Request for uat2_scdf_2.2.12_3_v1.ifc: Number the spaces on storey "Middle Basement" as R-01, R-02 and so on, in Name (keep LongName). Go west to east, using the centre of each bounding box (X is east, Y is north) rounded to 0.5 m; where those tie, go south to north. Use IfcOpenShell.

First a look at what the model holds.

```python
import ifcopenshell
import ifcopenshell.util.element
import ifcopenshell.util.placement

model = ifcopenshell.open("uat2_scdf_2.2.12_3_v1.ifc")
print(model.schema)
storey = next(s for s in model.by_type("IfcBuildingStorey") if s.Name == "Middle Basement")
spaces = [e for e in ifcopenshell.util.element.get_decomposition(storey) if e.is_a("IfcSpace")]
for e in sorted(spaces, key=lambda e: e.id()):
    origin = ifcopenshell.util.placement.get_local_placement(e.ObjectPlacement)[:3, 3]
    print(e.id(), e.Name, e.LongName, origin.round(2) + 0.0, sep=" | ")
```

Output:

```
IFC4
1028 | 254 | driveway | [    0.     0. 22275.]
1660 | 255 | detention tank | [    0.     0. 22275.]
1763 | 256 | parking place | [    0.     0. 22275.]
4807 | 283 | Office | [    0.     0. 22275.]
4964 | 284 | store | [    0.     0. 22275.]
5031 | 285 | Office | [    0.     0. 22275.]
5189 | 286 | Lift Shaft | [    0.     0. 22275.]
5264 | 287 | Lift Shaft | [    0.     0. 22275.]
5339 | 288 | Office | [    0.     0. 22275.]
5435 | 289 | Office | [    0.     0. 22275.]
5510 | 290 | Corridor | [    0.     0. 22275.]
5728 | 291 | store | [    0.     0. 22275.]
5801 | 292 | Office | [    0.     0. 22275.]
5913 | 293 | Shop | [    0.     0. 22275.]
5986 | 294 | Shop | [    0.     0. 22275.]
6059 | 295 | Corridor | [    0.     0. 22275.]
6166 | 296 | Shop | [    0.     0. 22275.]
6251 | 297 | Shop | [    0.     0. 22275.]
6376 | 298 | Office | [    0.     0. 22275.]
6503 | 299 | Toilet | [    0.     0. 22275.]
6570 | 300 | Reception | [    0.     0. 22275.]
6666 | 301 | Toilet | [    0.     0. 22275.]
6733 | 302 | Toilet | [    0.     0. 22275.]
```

```python
import ifcopenshell
import ifcopenshell.geom
import ifcopenshell.util.element
import ifcopenshell.util.shape

model = ifcopenshell.open("uat2_scdf_2.2.12_3_v1.ifc")
settings = ifcopenshell.geom.settings()
settings.set("use-world-coords", True)


def centre(element):
    shape = ifcopenshell.geom.create_shape(settings, element)
    return ifcopenshell.util.shape.get_bbox_centroid(shape.geometry)


storey = next(s for s in model.by_type("IfcBuildingStorey") if s.Name == "Middle Basement")
spaces = [e for e in ifcopenshell.util.element.get_decomposition(storey) if e.is_a("IfcSpace")]

# Insertion points can sit at a corner or the storey origin, so sort by the geometry (in metres).
centres = {e: centre(e) for e in spaces}
spaces.sort(key=lambda e: (round(centres[e][0] / 0.5), centres[e][1]))

for i, e in enumerate(spaces, start=1):
    number = f"R-{i:02d}"
    e.Name = number
    print(e.id(), number)

model.write("uat2_scdf_2.2.12_3_v1_v2.ifc")
```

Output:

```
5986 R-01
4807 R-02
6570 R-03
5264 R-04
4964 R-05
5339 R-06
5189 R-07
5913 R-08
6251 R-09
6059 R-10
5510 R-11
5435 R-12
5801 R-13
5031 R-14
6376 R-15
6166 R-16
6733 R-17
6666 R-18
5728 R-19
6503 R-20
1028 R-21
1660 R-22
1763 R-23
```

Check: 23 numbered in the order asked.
